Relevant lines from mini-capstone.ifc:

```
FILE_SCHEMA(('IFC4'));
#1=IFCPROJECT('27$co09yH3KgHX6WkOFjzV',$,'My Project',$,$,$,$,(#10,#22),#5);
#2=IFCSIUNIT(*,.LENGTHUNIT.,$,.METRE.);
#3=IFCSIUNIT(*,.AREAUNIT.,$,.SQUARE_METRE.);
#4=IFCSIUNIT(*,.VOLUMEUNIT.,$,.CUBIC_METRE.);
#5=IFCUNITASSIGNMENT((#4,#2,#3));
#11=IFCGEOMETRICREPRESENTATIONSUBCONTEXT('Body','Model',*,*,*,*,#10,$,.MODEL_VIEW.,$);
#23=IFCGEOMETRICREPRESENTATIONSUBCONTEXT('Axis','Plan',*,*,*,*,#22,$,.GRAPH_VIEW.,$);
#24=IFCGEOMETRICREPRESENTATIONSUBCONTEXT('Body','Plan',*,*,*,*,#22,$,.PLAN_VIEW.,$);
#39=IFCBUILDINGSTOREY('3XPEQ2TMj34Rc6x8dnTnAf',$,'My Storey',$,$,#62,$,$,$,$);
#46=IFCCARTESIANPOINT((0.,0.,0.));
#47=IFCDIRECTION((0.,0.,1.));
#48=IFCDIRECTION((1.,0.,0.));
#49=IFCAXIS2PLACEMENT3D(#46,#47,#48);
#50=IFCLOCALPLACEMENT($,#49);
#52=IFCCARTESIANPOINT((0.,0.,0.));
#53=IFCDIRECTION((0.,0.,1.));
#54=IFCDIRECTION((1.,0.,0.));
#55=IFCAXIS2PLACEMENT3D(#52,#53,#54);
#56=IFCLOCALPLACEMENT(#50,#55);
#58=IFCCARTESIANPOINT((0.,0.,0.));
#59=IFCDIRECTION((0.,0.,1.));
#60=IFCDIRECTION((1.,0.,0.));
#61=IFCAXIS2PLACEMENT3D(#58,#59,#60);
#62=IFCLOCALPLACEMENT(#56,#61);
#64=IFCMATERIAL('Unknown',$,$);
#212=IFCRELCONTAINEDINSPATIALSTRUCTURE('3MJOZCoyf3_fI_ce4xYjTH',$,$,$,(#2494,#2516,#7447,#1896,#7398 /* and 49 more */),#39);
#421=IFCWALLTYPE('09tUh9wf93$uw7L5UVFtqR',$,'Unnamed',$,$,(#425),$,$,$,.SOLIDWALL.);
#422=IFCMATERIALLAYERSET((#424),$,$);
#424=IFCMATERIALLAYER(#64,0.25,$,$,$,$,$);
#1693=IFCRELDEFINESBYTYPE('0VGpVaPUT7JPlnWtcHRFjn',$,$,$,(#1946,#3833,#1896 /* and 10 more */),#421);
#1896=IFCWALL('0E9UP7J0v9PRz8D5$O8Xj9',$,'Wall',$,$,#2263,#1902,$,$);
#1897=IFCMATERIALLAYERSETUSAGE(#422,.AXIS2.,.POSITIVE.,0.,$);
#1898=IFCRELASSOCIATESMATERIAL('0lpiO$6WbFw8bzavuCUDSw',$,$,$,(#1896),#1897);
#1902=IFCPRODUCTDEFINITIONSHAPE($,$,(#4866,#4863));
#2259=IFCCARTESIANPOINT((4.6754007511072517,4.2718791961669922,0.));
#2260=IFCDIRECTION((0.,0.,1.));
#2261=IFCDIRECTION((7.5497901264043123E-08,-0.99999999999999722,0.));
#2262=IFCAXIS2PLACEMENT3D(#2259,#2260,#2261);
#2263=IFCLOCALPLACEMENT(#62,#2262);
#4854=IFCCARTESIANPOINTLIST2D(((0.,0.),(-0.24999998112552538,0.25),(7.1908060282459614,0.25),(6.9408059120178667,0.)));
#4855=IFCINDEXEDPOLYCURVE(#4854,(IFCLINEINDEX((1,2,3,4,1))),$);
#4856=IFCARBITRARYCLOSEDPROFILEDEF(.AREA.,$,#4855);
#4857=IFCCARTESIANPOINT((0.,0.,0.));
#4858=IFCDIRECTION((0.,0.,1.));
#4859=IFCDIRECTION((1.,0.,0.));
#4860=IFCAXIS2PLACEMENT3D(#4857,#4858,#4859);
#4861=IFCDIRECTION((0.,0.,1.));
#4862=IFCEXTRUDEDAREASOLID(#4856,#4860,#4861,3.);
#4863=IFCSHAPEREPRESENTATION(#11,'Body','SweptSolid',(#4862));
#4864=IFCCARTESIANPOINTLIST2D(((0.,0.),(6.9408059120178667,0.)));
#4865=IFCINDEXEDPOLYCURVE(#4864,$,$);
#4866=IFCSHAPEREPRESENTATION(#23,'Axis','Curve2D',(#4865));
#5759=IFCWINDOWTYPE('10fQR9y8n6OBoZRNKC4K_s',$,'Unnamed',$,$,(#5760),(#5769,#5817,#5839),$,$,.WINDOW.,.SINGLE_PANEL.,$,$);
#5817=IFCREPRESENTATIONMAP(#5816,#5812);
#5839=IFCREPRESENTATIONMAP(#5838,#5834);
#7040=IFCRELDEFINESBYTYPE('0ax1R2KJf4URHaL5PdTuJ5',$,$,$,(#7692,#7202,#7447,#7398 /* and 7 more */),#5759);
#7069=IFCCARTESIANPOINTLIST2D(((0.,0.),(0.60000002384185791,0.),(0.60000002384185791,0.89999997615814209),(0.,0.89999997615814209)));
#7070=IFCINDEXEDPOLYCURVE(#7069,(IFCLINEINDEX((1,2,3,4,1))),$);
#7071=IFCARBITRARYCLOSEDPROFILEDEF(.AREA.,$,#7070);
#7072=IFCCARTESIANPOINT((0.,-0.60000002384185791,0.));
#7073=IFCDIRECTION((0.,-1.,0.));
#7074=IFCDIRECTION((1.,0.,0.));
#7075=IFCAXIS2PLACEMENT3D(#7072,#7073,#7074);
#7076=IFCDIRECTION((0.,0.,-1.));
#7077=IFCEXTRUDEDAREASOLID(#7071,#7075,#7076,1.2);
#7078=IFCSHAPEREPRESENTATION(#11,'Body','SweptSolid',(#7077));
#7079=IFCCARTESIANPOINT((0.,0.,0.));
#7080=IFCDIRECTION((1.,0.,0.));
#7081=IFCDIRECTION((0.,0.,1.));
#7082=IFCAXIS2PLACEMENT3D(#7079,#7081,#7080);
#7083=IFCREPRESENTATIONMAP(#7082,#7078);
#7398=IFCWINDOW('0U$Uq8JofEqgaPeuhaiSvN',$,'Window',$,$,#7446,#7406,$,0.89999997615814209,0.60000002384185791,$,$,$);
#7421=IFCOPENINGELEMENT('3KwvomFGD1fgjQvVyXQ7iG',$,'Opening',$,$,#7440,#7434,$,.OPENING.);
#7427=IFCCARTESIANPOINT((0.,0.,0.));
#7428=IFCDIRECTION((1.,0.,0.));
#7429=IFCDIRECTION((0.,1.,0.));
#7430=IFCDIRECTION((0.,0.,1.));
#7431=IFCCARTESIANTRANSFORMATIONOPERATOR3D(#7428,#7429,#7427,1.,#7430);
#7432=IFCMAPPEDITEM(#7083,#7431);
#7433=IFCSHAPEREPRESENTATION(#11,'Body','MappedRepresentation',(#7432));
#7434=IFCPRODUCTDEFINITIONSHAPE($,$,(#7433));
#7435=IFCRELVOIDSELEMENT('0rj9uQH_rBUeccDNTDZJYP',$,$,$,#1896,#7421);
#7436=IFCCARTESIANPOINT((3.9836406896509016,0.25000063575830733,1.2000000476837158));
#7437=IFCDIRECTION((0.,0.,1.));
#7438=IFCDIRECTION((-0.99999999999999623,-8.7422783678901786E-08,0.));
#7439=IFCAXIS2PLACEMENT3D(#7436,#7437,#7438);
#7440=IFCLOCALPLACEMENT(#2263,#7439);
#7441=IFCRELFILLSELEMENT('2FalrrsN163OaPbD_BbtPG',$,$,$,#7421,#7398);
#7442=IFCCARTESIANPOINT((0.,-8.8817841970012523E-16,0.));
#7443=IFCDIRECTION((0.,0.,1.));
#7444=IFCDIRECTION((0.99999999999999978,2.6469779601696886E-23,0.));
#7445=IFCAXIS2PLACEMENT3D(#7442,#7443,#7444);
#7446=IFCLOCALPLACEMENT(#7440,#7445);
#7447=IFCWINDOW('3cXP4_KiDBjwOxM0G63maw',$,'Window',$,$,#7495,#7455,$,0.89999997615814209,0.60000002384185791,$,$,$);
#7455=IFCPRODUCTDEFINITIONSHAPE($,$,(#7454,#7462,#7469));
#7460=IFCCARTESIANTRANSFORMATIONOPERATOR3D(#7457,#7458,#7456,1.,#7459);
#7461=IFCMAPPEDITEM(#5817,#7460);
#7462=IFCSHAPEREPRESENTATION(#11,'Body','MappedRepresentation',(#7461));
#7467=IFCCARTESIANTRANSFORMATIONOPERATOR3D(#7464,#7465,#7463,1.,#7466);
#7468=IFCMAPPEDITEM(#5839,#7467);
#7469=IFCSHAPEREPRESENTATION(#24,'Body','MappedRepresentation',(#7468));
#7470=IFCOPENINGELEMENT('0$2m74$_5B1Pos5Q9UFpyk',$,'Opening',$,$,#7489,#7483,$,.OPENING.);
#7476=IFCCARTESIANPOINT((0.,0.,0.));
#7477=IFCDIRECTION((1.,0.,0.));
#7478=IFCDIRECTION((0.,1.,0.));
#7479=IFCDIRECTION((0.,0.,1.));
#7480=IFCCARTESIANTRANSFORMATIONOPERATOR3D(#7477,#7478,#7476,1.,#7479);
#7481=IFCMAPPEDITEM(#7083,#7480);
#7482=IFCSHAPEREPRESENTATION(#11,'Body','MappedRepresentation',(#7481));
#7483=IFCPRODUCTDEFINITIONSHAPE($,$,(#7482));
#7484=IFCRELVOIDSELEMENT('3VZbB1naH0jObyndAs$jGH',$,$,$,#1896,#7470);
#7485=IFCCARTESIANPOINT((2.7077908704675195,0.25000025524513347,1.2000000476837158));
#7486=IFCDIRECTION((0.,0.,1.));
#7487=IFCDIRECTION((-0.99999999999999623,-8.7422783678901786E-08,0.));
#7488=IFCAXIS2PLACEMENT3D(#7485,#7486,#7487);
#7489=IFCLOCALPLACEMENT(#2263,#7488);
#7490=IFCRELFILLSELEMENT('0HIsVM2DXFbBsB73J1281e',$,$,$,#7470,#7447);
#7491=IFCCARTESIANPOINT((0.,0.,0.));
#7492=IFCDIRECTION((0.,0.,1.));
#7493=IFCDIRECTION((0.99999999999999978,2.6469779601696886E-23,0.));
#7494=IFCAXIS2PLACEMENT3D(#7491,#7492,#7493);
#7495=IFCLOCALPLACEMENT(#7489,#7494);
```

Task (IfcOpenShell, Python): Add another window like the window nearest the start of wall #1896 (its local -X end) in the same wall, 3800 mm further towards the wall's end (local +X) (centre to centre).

```python
import ifcopenshell
import ifcopenshell.api.feature
import ifcopenshell.api.geometry
import ifcopenshell.api.root
import ifcopenshell.geom
import ifcopenshell.util.element
import ifcopenshell.util.placement
import ifcopenshell.util.shape

model = ifcopenshell.open("mini-capstone.ifc")
settings = ifcopenshell.geom.settings()


def volume(element):
    """Net volume in cubic metres, openings subtracted."""
    shape = ifcopenshell.geom.create_shape(settings, element)
    return ifcopenshell.util.shape.get_volume(shape.geometry)


window = model.by_guid("3cXP4_KiDBjwOxM0G63maw")
opening = window.FillsVoids[0].RelatingOpeningElement
wall = opening.VoidsElements[0].RelatingBuildingElement
before = volume(wall)
shift = ifcopenshell.util.placement.get_local_placement(wall.ObjectPlacement)[:3, 0] * 3.8

# copy_class copies the void relationship, type, container and properties, but no geometry.
new_opening = ifcopenshell.api.root.copy_class(model, product=opening)
new_opening.Representation = ifcopenshell.util.element.copy_deep(
    model, opening.Representation, exclude=["IfcGeometricRepresentationContext", "IfcRepresentationMap"]
)
new_window = ifcopenshell.api.root.copy_class(model, product=window)
new_window.Representation = ifcopenshell.util.element.copy_deep(
    model, window.Representation, exclude=["IfcGeometricRepresentationContext", "IfcRepresentationMap"]
)
ifcopenshell.api.feature.add_filling(model, opening=new_opening, element=new_window)

for old, new in ((opening, new_opening), (window, new_window)):
    matrix = ifcopenshell.util.placement.get_local_placement(old.ObjectPlacement)
    matrix[:3, 3] += shift
    ifcopenshell.api.geometry.edit_object_placement(model, product=new, matrix=matrix, is_si=False)

after = volume(wall)

print(f"wall volume {before:.3f} -> {after:.3f} m3")

model.write("mini-capstone_updated.ifc")
```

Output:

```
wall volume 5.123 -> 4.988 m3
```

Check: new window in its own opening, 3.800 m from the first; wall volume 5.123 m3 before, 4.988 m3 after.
